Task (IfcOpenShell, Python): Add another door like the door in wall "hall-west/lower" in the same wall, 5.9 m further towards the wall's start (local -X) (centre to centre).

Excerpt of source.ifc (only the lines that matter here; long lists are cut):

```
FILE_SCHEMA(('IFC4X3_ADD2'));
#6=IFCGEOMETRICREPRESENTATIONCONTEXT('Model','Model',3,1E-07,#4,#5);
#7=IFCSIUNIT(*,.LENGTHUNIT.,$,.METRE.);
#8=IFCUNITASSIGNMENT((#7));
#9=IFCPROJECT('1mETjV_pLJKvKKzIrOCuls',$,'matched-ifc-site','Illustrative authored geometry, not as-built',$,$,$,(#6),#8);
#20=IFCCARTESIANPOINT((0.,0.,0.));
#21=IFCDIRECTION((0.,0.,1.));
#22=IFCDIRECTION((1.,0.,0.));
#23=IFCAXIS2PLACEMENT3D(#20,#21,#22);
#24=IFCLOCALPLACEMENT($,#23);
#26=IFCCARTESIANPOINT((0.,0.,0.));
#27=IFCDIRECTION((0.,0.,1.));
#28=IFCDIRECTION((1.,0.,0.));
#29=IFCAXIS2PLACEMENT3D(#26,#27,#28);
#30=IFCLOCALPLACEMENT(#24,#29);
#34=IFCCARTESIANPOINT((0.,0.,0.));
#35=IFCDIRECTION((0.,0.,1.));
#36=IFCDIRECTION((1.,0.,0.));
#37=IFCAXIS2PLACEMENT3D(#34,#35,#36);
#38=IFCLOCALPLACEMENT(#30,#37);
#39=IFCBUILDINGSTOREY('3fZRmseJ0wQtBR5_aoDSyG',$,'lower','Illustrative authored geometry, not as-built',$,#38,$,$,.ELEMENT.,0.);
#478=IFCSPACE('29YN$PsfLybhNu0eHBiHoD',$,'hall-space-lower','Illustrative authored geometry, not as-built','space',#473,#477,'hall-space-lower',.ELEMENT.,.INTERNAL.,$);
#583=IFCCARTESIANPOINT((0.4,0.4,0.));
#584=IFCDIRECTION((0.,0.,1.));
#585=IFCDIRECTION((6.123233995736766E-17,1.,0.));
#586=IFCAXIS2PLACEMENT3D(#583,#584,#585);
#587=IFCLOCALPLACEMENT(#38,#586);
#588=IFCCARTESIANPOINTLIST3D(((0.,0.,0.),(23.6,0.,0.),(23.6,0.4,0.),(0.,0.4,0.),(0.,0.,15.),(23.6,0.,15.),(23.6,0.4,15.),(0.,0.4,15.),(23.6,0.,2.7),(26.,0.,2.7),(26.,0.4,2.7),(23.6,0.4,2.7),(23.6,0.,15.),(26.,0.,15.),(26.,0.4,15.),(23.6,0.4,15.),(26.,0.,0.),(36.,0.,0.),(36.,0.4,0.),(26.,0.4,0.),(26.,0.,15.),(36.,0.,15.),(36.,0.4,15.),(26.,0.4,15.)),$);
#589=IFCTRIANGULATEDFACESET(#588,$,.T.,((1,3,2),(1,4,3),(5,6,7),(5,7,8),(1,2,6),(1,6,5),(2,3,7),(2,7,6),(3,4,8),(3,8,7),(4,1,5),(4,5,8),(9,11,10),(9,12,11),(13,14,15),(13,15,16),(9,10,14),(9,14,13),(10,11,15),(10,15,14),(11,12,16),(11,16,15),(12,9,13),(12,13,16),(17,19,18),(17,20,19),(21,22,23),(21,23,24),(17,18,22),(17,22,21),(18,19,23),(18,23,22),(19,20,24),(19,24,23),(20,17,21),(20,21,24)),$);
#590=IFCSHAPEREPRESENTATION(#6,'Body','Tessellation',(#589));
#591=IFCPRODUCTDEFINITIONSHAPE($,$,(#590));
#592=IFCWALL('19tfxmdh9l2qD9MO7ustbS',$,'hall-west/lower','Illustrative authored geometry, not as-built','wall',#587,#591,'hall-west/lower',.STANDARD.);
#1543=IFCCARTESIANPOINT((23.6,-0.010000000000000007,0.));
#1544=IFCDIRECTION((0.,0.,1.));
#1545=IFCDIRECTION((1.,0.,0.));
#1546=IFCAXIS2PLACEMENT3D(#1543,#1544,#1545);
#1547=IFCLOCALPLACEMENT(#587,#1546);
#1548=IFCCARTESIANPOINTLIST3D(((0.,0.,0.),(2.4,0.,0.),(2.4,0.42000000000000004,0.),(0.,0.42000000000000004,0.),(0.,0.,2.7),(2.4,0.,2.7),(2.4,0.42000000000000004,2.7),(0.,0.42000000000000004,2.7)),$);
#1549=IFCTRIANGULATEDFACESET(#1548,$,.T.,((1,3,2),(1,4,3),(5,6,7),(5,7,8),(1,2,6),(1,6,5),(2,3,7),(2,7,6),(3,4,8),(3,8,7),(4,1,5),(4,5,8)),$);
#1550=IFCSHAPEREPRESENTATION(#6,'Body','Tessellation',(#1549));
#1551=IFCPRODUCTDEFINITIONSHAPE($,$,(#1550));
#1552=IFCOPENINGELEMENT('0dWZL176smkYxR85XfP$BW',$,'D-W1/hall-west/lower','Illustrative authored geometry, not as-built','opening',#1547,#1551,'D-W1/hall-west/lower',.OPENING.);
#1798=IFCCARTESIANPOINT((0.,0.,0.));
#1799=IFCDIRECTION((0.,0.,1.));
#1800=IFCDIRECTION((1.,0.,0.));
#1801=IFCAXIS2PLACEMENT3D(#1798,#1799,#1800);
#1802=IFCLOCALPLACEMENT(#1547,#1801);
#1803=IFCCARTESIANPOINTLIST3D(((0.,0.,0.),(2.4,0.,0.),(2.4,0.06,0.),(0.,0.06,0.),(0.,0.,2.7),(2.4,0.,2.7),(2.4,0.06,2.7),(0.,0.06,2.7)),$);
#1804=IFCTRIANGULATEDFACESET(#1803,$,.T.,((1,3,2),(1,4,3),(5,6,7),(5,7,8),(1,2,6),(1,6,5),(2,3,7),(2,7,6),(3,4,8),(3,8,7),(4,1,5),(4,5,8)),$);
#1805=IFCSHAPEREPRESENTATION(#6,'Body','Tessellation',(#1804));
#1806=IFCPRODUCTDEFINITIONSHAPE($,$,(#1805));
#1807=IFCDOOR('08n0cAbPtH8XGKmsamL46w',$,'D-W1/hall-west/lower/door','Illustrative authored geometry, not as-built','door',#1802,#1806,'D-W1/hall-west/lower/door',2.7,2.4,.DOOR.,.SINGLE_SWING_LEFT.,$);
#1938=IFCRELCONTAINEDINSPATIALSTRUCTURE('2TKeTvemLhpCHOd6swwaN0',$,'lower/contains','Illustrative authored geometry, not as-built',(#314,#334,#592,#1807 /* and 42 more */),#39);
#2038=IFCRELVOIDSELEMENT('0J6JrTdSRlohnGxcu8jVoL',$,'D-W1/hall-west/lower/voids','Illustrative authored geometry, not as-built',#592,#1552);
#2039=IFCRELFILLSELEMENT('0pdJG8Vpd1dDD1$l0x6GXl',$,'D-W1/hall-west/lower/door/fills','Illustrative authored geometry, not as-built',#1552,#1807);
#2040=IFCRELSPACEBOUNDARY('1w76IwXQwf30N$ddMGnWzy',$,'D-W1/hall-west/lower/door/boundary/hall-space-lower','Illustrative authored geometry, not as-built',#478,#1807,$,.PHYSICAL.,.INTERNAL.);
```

```python
import ifcopenshell
import ifcopenshell.api.feature
import ifcopenshell.api.geometry
import ifcopenshell.api.root
import ifcopenshell.geom
import ifcopenshell.util.element
import ifcopenshell.util.placement
import ifcopenshell.util.shape
import ifcopenshell.util.unit

model = ifcopenshell.open("source.ifc")
unit_scale = ifcopenshell.util.unit.calculate_unit_scale(model)
settings = ifcopenshell.geom.settings()


def volume(element):
    """Net volume in cubic metres, openings subtracted."""
    shape = ifcopenshell.geom.create_shape(settings, element)
    return ifcopenshell.util.shape.get_volume(shape.geometry)


door = model.by_guid("08n0cAbPtH8XGKmsamL46w")
opening = door.FillsVoids[0].RelatingOpeningElement
wall = opening.VoidsElements[0].RelatingBuildingElement
before = volume(wall)
shift = ifcopenshell.util.placement.get_local_placement(wall.ObjectPlacement)[:3, 0] * -5.9 / unit_scale

# copy_class copies the void relationship, type, container and properties, but no geometry.
new_opening = ifcopenshell.api.root.copy_class(model, product=opening)
new_opening.Representation = ifcopenshell.util.element.copy_deep(
    model, opening.Representation, exclude=["IfcGeometricRepresentationContext", "IfcRepresentationMap"]
)
new_opening.Tag = None
new_door = ifcopenshell.api.root.copy_class(model, product=door)
new_door.Representation = ifcopenshell.util.element.copy_deep(
    model, door.Representation, exclude=["IfcGeometricRepresentationContext", "IfcRepresentationMap"]
)
new_door.Tag = None
ifcopenshell.api.feature.add_filling(model, opening=new_opening, element=new_door)

for old, new in ((opening, new_opening), (door, new_door)):
    matrix = ifcopenshell.util.placement.get_local_placement(old.ObjectPlacement)
    matrix[:3, 3] += shift
    ifcopenshell.api.geometry.edit_object_placement(model, product=new, matrix=matrix, is_si=False)

after = volume(wall)

print(f"wall volume {before:.3f} -> {after:.3f} m3")

model.write("source_rev.ifc")
```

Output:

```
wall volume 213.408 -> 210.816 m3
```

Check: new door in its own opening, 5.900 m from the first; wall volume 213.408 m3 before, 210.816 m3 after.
